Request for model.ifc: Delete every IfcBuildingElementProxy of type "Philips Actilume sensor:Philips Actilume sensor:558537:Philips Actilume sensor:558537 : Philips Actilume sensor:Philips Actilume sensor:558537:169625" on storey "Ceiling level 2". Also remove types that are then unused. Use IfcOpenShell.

First a look at what the model holds.

```python
import ifcopenshell
import ifcopenshell.util.element

model = ifcopenshell.open("model.ifc")
print(model.schema)
storey = next(s for s in model.by_type("IfcBuildingStorey") if s.Name == "Ceiling level 2")
proxies = [e for e in ifcopenshell.util.element.get_decomposition(storey) if e.is_a("IfcBuildingElementProxy")]
seen = {}
for e in proxies:
    element_type = ifcopenshell.util.element.get_type(e)
    name = element_type.Name if element_type not in (None, e) else None
    seen[name] = seen.get(name, 0) + 1
for name, count in sorted(seen.items(), key=str):
    print(count, "x", name)
```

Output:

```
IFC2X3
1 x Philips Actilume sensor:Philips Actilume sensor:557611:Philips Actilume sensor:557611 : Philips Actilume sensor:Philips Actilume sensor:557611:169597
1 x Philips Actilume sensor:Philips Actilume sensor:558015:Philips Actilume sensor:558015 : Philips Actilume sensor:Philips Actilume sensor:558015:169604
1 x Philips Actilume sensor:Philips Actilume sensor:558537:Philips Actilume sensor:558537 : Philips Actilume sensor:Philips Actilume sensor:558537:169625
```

```python
import ifcopenshell
import ifcopenshell.api.root
import ifcopenshell.util.element

model = ifcopenshell.open("model.ifc")

storey = next(s for s in model.by_type("IfcBuildingStorey") if s.Name == "Ceiling level 2")
proxies = [e for e in ifcopenshell.util.element.get_decomposition(storey) if e.is_a("IfcBuildingElementProxy")]
targets = [e for e in proxies if (t := ifcopenshell.util.element.get_type(e)) not in (None, e) and t.Name == "Philips Actilume sensor:Philips Actilume sensor:558537:Philips Actilume sensor:558537 : Philips Actilume sensor:Philips Actilume sensor:558537:169625"]
types = {ifcopenshell.util.element.get_type(e) for e in targets} - {None, *targets}

for e in targets:
    ifcopenshell.api.root.remove_product(model, product=e)
print(len(targets), "removed")

unused = [t for t in types if not ifcopenshell.util.element.get_types(t)]
for t in unused:
    ifcopenshell.api.root.remove_product(model, product=t)
print(len(unused), "unused types removed")

model.write("model_edited.ifc")
```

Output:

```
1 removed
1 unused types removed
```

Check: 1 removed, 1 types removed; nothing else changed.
